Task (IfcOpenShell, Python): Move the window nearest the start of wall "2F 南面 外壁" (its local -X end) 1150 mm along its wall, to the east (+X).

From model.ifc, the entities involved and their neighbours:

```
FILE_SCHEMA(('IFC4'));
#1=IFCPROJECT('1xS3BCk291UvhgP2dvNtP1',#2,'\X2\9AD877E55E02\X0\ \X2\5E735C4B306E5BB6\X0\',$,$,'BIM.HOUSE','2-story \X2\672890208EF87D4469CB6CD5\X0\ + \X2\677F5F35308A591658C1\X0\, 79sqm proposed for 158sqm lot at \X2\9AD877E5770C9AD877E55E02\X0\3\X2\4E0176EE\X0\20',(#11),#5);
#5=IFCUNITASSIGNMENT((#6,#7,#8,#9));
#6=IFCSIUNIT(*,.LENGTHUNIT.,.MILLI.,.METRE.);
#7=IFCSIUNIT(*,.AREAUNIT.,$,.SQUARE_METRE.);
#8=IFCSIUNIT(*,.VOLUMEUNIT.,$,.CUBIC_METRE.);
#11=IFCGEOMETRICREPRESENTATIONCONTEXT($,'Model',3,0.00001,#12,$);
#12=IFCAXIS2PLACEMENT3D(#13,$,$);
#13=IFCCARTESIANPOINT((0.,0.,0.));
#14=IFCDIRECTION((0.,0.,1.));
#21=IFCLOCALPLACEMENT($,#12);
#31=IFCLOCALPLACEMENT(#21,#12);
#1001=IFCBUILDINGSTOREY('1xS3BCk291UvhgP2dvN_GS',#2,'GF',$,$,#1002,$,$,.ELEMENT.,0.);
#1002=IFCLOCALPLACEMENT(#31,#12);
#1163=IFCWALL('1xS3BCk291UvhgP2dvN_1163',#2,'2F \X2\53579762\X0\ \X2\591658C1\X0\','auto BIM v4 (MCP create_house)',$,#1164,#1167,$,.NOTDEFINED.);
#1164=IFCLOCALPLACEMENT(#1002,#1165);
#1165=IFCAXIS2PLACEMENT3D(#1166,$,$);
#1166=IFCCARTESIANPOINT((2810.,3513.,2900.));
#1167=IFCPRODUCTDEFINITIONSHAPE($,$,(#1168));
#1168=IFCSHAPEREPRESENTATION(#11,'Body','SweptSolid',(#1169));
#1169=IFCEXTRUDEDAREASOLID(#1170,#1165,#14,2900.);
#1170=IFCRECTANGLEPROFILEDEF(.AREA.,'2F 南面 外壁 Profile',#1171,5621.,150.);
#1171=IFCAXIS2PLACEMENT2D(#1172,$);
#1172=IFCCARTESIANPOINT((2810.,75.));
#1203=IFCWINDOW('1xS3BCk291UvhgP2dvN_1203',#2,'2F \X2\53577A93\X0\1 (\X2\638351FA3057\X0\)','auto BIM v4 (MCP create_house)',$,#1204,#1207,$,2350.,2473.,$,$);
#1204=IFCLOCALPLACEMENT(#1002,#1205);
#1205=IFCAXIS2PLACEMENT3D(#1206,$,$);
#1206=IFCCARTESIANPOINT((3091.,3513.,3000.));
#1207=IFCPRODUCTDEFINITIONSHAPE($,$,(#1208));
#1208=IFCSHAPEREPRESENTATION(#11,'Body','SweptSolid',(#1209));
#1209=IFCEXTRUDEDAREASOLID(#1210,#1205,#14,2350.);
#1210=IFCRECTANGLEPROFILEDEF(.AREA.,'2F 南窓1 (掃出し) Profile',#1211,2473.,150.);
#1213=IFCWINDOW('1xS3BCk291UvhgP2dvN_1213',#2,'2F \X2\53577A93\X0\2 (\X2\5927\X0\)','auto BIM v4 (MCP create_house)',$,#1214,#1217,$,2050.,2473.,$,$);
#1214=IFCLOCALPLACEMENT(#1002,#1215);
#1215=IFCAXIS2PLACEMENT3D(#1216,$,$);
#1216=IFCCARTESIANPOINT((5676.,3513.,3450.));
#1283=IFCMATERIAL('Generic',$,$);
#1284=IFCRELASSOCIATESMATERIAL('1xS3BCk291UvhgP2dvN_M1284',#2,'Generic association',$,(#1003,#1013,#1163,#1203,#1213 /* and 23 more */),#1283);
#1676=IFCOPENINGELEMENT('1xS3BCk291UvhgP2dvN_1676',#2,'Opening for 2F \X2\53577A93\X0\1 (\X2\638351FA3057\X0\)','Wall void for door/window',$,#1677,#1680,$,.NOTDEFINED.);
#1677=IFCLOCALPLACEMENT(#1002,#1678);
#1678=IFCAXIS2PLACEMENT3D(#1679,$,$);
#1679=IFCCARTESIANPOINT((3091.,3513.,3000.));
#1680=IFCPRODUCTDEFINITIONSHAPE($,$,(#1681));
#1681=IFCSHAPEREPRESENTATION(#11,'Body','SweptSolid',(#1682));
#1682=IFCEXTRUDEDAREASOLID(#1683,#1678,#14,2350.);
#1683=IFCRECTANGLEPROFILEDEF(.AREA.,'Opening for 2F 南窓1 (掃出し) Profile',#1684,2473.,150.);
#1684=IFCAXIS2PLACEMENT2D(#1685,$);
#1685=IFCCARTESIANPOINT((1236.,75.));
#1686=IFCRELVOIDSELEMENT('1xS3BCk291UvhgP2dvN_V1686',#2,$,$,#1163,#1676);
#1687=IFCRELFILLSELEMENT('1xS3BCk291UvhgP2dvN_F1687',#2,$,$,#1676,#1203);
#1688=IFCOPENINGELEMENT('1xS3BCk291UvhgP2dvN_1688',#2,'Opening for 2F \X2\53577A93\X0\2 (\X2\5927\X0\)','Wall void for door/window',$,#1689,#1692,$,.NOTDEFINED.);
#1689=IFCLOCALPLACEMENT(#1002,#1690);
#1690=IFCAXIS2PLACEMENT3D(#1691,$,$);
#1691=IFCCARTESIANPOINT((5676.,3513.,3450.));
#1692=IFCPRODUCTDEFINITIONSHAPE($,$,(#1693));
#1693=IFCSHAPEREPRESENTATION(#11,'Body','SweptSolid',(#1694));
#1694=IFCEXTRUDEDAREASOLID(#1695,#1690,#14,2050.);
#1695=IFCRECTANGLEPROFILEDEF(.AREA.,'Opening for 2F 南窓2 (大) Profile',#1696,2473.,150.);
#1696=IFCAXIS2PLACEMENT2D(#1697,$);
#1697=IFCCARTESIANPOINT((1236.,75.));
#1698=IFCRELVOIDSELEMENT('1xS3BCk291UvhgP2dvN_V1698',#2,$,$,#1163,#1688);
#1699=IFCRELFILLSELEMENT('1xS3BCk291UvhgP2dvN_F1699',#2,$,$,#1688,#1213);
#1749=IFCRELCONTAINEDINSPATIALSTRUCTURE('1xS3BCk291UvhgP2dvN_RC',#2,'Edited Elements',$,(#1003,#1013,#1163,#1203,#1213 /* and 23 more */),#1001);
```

```python
import ifcopenshell
import ifcopenshell.api.geometry
import ifcopenshell.util.placement
import ifcopenshell.util.unit

model = ifcopenshell.open("model.ifc")
unit_scale = ifcopenshell.util.unit.calculate_unit_scale(model)

window = model.by_id(1203)
opening = window.FillsVoids[0].RelatingOpeningElement
wall = opening.VoidsElements[0].RelatingBuildingElement

wall_matrix = ifcopenshell.util.placement.get_local_placement(wall.ObjectPlacement)
shift = wall_matrix[:3, 0] * 1.15 / unit_scale
before = ifcopenshell.util.placement.get_local_placement(window.ObjectPlacement)[:3, 3].copy()

# The window is not placed relative to its opening, so move both.
for product in (opening, window):
    matrix = ifcopenshell.util.placement.get_local_placement(product.ObjectPlacement)
    matrix[:3, 3] += shift
    ifcopenshell.api.geometry.edit_object_placement(model, product=product, matrix=matrix, is_si=False)

after = ifcopenshell.util.placement.get_local_placement(window.ObjectPlacement)[:3, 3]
print("window moved by", (after - before).round(3) + 0.0)

model.write("model_rev.ifc")
```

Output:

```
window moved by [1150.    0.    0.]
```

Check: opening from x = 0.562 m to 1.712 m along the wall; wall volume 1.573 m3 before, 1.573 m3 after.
